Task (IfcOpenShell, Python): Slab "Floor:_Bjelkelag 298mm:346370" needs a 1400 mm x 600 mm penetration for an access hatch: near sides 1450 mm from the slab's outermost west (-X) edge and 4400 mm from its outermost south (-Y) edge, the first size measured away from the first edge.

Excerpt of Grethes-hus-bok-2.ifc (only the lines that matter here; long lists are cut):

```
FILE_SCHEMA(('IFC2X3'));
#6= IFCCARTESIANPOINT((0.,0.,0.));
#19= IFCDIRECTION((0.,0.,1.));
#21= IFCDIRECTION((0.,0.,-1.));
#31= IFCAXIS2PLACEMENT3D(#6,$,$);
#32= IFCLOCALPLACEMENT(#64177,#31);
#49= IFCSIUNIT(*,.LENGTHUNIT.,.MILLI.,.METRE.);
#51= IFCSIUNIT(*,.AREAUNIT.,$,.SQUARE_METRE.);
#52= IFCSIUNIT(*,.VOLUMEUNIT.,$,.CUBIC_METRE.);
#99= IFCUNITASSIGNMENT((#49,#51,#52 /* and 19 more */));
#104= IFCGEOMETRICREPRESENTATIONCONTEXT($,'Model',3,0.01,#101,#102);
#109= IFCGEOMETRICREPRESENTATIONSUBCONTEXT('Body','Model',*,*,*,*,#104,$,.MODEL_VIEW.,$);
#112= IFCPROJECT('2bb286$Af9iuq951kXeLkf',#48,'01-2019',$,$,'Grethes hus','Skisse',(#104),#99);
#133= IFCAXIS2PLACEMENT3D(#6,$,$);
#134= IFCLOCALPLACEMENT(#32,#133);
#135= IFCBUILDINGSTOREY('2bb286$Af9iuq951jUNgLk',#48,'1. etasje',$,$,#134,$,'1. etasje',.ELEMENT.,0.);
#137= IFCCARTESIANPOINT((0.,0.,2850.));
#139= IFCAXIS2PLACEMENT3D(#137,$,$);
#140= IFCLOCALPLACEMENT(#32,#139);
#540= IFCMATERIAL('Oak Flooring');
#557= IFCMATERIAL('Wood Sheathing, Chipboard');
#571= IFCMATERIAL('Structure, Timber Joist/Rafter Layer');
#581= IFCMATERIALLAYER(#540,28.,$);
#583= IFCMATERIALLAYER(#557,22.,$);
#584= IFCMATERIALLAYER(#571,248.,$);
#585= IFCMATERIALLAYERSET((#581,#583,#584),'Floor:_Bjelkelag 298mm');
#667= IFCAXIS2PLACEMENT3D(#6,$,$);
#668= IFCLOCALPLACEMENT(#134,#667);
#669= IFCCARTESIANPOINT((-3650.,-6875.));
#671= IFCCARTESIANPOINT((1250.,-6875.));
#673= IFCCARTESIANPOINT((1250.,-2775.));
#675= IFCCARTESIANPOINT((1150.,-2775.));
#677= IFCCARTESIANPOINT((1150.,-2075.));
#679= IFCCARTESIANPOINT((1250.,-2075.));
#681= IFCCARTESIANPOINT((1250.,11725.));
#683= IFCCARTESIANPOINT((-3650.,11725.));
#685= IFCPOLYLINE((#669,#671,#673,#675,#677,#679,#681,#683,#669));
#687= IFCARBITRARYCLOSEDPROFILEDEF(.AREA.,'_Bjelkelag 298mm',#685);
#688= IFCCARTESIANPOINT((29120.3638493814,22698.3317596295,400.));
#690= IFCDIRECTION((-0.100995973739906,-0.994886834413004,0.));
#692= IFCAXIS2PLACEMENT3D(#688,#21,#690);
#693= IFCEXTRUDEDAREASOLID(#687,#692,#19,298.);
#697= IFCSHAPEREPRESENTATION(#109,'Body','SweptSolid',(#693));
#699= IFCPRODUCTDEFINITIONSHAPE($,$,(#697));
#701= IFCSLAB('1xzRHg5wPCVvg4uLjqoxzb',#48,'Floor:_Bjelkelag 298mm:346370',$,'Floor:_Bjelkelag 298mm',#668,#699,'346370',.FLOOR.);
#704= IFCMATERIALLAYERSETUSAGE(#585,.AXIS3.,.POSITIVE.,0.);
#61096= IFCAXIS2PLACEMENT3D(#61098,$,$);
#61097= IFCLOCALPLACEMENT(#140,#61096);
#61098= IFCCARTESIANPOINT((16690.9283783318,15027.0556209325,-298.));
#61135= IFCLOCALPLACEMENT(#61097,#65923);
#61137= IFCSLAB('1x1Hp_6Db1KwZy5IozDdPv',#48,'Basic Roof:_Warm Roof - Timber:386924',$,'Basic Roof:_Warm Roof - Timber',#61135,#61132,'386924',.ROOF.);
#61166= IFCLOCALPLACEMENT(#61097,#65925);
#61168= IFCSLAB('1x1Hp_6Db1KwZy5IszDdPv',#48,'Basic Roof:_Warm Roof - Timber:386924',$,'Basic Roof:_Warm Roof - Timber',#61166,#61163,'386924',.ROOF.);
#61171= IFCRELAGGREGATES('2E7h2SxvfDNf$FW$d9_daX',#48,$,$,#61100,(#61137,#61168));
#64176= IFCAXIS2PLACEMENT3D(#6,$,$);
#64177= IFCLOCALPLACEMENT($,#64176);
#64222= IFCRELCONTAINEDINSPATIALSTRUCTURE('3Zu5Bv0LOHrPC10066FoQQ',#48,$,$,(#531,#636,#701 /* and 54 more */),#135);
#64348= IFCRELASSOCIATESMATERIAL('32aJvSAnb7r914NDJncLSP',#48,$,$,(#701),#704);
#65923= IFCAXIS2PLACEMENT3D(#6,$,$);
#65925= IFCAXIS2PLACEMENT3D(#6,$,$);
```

```python
import numpy as np
import ifcopenshell
import ifcopenshell.api.feature
import ifcopenshell.api.geometry
import ifcopenshell.api.root
import ifcopenshell.geom
import ifcopenshell.util.placement
import ifcopenshell.util.representation
import ifcopenshell.util.shape
import ifcopenshell.util.unit

model = ifcopenshell.open("Grethes-hus-bok-2.ifc")
unit_scale = ifcopenshell.util.unit.calculate_unit_scale(model)
settings = ifcopenshell.geom.settings()


def volume(element):
    """Net volume in cubic metres, openings subtracted."""
    shape = ifcopenshell.geom.create_shape(settings, element)
    return ifcopenshell.util.shape.get_volume(shape.geometry)


slab = model.by_guid("1xzRHg5wPCVvg4uLjqoxzb")
before = volume(slab)

# Extent in the slab's own axes, in metres. The edges named are its -X and -Y sides.
slab_shape = ifcopenshell.geom.create_shape(settings, slab)
vertices = ifcopenshell.util.shape.get_vertices(slab_shape.geometry)
x_min, y_min, bottom = vertices.min(axis=0)
top = vertices[:, 2].max()

opening = ifcopenshell.api.root.create_entity(model, ifc_class="IfcOpeningElement", name="Access hatch opening")
context = ifcopenshell.util.representation.get_context(model, "Model", "Body", "MODEL_VIEW")
width, depth = 1.4, 0.6
outline = [(0.0, 0.0), (width, 0.0), (width, depth), (0.0, depth), (0.0, 0.0)]
# Overshoot both faces by 50 mm so the cut is clean.
shape = ifcopenshell.api.geometry.add_slab_representation(
    model, context=context, depth=top - bottom + 0.1, polyline=outline
)
ifcopenshell.api.geometry.assign_representation(model, product=opening, representation=shape)

matrix = ifcopenshell.util.placement.get_local_placement(slab.ObjectPlacement)
matrix[:, 3] = matrix @ np.append(np.array([x_min + 1.45, y_min + 4.4, bottom - 0.05]) / unit_scale, 1.0)
ifcopenshell.api.geometry.edit_object_placement(model, product=opening, matrix=matrix, is_si=False)
ifcopenshell.api.feature.add_feature(model, feature=opening, element=slab)

after = volume(slab)

print(f"slab volume {before:.3f} -> {after:.3f} m3")

model.write("Grethes-hus-bok-2-out.ifc")
```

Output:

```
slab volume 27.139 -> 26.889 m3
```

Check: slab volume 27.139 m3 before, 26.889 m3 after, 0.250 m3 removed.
